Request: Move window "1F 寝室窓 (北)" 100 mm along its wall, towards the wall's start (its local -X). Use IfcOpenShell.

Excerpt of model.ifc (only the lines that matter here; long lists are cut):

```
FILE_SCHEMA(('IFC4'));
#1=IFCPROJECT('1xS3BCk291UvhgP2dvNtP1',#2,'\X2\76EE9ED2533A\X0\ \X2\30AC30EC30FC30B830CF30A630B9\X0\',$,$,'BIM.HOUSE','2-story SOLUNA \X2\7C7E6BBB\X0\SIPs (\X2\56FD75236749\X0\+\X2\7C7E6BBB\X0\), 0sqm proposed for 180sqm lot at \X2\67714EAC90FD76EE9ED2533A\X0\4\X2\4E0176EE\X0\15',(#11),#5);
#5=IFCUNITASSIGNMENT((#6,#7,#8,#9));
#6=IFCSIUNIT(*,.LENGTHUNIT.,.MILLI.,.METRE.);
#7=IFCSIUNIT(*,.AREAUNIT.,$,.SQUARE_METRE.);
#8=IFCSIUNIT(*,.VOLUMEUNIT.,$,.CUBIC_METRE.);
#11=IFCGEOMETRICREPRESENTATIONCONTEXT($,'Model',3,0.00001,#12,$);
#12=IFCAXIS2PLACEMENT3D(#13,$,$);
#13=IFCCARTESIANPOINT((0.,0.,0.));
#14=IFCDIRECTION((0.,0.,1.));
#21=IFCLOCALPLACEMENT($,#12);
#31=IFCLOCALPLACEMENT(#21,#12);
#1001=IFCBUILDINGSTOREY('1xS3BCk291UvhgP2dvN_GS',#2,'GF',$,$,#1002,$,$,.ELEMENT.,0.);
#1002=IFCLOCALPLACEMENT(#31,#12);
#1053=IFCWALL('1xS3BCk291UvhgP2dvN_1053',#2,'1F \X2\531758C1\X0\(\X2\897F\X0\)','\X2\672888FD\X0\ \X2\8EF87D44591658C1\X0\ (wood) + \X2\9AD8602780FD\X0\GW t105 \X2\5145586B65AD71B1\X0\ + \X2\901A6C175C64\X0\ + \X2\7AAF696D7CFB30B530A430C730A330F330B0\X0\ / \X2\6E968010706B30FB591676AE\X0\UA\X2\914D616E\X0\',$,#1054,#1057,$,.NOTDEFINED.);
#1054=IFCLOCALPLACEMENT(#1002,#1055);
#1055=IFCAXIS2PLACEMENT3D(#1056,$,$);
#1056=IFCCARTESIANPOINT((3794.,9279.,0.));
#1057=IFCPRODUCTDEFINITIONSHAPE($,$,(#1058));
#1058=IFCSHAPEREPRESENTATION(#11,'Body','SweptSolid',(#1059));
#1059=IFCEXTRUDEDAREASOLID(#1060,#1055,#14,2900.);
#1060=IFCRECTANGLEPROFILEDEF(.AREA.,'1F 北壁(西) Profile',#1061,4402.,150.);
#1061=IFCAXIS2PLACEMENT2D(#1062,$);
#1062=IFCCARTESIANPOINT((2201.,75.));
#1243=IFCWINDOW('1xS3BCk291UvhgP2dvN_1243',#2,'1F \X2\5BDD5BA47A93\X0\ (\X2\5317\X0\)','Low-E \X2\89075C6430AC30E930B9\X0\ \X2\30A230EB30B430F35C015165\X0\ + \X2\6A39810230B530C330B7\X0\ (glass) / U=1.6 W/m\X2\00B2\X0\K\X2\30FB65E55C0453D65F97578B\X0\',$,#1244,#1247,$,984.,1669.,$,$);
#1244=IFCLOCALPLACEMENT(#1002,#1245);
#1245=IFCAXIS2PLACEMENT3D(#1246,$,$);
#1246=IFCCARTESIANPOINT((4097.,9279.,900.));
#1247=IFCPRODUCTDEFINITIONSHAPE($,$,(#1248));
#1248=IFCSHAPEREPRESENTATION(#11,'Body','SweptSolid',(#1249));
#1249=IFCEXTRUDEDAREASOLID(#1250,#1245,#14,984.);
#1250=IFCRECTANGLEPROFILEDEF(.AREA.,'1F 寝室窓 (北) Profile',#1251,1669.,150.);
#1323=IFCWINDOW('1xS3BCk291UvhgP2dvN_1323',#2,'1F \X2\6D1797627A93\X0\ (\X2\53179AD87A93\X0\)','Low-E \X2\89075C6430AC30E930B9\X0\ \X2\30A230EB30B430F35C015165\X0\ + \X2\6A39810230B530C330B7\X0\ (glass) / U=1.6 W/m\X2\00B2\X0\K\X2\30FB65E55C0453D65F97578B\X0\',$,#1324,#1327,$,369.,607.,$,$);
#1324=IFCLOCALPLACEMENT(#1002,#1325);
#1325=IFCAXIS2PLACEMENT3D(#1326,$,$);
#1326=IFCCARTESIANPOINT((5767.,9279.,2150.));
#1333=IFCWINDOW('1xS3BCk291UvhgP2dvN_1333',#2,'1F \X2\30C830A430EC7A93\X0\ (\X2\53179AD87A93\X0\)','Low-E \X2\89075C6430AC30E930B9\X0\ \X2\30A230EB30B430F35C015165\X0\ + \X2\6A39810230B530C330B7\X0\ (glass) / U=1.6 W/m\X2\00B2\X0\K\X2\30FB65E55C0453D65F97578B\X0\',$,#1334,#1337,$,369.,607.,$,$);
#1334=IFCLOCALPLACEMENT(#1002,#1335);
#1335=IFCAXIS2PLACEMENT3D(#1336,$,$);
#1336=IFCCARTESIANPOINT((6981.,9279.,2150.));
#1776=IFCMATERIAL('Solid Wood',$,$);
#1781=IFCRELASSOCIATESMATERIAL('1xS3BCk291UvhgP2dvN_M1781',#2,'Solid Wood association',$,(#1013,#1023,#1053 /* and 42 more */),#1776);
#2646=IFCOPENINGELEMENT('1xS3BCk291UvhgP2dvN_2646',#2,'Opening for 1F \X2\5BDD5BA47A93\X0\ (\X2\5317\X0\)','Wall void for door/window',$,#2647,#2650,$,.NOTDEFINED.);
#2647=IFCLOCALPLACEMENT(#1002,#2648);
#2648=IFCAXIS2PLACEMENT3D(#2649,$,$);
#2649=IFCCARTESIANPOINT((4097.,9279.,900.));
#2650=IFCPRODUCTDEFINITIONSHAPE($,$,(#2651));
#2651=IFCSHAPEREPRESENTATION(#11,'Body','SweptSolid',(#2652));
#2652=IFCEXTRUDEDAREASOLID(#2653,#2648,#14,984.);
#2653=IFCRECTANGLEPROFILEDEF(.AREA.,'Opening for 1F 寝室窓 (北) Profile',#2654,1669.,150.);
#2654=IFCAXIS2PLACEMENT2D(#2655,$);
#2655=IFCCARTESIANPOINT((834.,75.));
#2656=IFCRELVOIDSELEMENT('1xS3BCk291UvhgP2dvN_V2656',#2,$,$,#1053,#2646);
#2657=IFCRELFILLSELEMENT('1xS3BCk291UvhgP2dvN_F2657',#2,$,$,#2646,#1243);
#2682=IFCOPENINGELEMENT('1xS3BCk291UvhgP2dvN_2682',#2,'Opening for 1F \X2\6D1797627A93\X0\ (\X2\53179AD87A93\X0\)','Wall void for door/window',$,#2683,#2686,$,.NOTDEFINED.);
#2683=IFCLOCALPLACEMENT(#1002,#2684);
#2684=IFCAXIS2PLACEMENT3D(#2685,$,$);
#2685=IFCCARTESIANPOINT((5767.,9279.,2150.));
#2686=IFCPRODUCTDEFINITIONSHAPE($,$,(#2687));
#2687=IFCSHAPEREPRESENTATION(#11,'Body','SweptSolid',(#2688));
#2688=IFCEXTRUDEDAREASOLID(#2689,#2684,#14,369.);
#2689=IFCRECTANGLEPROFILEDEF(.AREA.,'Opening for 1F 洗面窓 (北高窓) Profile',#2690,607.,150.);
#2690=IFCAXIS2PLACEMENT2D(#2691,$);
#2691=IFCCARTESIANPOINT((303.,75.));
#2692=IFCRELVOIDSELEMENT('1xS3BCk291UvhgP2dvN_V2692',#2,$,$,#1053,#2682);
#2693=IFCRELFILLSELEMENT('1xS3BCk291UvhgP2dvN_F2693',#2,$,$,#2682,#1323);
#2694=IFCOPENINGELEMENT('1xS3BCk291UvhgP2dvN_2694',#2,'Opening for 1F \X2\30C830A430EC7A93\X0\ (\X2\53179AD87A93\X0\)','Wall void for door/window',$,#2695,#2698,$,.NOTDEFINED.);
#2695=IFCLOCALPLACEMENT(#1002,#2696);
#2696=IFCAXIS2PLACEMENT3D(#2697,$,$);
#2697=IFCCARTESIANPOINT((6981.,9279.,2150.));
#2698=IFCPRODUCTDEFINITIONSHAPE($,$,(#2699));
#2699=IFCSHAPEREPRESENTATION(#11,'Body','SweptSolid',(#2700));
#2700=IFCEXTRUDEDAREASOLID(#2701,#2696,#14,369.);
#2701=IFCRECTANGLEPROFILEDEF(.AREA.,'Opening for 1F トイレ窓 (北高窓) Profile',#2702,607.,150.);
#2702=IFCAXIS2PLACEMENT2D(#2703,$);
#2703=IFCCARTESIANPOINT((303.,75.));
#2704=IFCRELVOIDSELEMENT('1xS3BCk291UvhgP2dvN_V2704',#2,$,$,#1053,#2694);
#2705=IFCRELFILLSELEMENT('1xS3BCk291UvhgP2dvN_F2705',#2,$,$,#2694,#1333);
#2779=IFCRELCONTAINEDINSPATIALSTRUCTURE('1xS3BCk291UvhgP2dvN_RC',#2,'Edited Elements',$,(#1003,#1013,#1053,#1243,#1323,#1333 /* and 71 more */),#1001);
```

```python
import ifcopenshell
import ifcopenshell.api.geometry
import ifcopenshell.util.placement
import ifcopenshell.util.unit

model = ifcopenshell.open("model.ifc")
unit_scale = ifcopenshell.util.unit.calculate_unit_scale(model)

window = model.by_id(1243)
opening = window.FillsVoids[0].RelatingOpeningElement
wall = opening.VoidsElements[0].RelatingBuildingElement

wall_matrix = ifcopenshell.util.placement.get_local_placement(wall.ObjectPlacement)
shift = wall_matrix[:3, 0] * -0.1 / unit_scale
before = ifcopenshell.util.placement.get_local_placement(window.ObjectPlacement)[:3, 3].copy()

# The window is not placed relative to its opening, so move both.
for product in (opening, window):
    matrix = ifcopenshell.util.placement.get_local_placement(product.ObjectPlacement)
    matrix[:3, 3] += shift
    ifcopenshell.api.geometry.edit_object_placement(model, product=product, matrix=matrix, is_si=False)

after = ifcopenshell.util.placement.get_local_placement(window.ObjectPlacement)[:3, 3]
print("window moved by", (after - before).round(3) + 0.0)

model.write("model_v2.ifc")
```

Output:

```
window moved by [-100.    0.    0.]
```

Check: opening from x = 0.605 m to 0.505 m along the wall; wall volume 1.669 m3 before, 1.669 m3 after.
